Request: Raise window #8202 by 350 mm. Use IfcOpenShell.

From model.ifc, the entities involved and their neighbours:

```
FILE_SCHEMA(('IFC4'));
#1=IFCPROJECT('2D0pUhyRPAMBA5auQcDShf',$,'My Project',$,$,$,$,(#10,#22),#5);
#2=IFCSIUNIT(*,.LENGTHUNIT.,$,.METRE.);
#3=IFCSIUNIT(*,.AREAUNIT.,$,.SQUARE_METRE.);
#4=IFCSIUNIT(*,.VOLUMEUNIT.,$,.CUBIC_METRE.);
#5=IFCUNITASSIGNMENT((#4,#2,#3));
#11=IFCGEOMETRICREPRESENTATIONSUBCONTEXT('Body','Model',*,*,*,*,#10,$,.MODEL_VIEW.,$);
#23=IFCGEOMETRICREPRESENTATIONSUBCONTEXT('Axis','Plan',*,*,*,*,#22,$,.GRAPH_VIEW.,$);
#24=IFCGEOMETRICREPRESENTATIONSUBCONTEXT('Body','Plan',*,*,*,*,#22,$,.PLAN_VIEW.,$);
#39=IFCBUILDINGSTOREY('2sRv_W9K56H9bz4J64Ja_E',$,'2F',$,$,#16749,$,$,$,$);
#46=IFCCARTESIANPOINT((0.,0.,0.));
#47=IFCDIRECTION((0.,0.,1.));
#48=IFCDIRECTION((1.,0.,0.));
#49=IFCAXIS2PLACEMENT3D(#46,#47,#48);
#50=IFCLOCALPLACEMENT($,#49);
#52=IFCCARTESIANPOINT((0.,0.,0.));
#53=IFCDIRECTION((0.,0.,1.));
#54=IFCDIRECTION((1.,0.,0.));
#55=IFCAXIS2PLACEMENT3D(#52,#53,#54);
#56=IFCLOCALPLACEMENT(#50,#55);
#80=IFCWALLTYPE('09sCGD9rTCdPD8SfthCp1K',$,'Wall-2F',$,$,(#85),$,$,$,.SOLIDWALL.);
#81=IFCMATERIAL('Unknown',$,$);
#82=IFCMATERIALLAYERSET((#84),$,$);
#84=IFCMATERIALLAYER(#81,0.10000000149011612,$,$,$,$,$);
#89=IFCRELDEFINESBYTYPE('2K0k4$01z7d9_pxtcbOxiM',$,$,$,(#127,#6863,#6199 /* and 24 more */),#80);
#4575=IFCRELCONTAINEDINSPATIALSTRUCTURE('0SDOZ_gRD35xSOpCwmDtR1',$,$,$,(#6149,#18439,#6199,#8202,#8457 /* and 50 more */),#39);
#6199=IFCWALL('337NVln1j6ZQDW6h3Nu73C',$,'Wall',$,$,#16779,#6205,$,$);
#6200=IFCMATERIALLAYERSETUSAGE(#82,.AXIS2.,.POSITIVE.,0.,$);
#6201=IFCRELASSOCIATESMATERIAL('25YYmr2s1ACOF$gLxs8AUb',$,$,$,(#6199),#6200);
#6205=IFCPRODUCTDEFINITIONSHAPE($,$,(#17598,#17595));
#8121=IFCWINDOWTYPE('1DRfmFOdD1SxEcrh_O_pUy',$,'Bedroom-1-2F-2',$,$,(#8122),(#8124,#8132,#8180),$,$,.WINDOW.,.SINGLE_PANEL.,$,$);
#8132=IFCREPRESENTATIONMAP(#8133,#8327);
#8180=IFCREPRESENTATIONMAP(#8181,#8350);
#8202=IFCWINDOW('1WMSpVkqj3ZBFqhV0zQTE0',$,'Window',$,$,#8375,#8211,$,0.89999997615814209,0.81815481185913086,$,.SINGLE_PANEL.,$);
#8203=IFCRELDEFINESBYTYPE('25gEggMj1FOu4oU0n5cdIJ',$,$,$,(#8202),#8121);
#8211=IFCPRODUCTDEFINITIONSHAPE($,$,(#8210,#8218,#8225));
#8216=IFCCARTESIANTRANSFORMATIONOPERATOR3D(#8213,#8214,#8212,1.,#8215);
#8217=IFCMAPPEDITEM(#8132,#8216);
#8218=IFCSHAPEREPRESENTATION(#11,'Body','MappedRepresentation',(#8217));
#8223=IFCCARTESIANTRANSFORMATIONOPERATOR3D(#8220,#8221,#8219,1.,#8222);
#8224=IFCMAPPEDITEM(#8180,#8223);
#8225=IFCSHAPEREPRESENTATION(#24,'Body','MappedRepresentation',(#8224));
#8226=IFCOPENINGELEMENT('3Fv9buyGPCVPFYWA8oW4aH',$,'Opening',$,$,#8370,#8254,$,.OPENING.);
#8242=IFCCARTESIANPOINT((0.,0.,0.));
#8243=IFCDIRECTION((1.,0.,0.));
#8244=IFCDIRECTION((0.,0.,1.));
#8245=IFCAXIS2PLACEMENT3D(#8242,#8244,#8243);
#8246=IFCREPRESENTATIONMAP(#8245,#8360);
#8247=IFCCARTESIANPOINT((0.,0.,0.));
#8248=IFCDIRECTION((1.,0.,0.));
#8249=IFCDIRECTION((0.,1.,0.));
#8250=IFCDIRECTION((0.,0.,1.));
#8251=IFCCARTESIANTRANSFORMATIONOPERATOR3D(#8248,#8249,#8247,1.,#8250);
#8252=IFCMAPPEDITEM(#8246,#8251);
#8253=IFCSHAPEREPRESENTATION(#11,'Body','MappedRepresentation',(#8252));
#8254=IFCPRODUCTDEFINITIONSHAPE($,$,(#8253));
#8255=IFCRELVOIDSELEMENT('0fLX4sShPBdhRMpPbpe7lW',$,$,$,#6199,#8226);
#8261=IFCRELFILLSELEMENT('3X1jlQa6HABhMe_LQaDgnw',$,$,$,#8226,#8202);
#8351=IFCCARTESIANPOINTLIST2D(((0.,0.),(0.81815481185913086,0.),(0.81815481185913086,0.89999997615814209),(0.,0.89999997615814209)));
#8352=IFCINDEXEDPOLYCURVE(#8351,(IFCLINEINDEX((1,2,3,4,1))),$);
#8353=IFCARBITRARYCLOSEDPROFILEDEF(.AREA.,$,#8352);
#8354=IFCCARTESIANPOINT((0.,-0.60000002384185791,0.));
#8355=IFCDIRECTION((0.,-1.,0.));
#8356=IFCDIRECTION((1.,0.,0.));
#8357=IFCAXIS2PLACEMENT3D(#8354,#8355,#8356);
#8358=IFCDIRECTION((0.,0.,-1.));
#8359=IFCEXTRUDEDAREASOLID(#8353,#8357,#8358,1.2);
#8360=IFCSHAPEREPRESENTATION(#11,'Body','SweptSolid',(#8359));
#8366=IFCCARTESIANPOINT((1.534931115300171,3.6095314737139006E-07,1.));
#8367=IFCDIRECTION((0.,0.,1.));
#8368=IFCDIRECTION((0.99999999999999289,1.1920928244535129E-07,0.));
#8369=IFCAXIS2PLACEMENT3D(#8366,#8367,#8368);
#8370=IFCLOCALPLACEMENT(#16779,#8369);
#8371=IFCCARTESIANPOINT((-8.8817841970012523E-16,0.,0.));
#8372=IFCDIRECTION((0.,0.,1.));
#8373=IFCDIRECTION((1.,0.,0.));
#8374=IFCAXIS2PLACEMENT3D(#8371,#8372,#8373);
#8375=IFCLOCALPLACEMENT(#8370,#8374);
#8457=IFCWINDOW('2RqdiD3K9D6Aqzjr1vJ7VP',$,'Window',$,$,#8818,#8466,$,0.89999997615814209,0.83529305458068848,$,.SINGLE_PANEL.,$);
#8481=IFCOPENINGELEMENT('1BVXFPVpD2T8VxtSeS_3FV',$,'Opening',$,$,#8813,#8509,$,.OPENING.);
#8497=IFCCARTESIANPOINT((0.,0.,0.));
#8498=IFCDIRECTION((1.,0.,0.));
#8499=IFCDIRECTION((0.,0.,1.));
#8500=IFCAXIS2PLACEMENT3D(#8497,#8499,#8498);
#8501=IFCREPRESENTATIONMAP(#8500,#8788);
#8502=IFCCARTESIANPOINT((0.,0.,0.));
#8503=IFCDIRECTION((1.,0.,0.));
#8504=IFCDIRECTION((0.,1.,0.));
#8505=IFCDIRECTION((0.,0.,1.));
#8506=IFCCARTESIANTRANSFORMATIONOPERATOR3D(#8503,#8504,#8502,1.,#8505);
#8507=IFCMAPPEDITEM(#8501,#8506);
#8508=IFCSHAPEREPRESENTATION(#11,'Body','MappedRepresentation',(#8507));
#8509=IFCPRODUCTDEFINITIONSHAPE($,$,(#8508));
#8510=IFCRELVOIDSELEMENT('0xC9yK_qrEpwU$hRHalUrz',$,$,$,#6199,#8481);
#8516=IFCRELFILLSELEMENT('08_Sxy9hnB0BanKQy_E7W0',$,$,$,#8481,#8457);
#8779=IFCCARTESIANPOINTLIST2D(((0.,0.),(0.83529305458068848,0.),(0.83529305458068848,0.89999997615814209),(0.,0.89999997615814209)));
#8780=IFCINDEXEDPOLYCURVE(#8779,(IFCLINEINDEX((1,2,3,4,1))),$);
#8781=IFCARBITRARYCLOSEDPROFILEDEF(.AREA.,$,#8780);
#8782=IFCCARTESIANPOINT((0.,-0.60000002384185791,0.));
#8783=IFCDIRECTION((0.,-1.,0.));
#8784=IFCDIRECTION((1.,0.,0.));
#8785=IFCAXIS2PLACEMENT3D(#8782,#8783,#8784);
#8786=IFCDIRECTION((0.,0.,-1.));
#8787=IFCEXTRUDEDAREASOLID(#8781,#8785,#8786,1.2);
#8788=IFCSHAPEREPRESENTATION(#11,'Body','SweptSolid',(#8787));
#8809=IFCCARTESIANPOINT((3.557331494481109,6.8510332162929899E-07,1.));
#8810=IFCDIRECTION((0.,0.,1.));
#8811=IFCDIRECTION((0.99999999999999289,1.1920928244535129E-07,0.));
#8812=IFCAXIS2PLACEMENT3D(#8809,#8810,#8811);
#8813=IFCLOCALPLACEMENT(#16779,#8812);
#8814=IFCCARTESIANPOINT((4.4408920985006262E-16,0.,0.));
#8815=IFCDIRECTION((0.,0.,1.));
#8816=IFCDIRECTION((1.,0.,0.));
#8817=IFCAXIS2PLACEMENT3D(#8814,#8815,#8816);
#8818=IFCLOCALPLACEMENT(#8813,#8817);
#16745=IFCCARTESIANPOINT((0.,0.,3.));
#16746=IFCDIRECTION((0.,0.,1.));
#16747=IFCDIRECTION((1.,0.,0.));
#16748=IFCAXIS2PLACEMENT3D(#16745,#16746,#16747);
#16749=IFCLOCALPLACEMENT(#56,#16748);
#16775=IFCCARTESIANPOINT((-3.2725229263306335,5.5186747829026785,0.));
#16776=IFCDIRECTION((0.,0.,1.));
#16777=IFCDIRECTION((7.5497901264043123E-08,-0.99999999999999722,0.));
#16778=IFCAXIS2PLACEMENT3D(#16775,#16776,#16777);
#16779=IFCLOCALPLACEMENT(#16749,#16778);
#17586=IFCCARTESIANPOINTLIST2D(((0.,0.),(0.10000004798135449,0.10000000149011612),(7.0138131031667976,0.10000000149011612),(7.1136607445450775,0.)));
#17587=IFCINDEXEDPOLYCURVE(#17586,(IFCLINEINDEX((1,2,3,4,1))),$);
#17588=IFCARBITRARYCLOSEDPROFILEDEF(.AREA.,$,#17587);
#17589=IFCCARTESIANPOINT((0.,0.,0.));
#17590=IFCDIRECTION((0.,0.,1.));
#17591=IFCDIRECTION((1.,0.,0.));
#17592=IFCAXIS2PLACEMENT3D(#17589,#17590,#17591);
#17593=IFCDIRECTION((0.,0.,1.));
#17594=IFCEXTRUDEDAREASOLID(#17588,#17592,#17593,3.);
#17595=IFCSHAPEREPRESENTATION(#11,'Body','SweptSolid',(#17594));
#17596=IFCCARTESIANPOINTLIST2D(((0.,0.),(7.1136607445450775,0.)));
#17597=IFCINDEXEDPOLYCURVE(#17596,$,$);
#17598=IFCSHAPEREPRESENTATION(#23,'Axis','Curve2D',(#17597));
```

```python
import numpy as np
import ifcopenshell
import ifcopenshell.api.geometry
import ifcopenshell.util.placement
import ifcopenshell.util.unit

model = ifcopenshell.open("model.ifc")
unit_scale = ifcopenshell.util.unit.calculate_unit_scale(model)

window = model.by_guid("1WMSpVkqj3ZBFqhV0zQTE0")
opening = window.FillsVoids[0].RelatingOpeningElement
dz = 0.35 / unit_scale

shift = np.array([0.0, 0.0, dz])
# The window is placed relative to its opening, so it follows when the opening moves.
matrix = ifcopenshell.util.placement.get_local_placement(opening.ObjectPlacement)
matrix[:3, 3] += shift
ifcopenshell.api.geometry.edit_object_placement(
    model, product=opening, matrix=matrix, is_si=False, should_transform_children=True
)

print(f"moved by {dz * unit_scale:+.3f} m")

model.write("model_updated.ifc")
```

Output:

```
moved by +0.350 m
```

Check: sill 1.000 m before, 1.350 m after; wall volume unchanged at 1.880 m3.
